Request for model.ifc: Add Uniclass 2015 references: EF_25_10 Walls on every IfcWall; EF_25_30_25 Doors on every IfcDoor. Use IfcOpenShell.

First a look at what the model holds.

```python
import ifcopenshell

model = ifcopenshell.open("model.ifc")
print(model.schema)
print("classifications:", [c.Name for c in model.by_type("IfcClassification")])
for ifc_class in ("IfcDoor", "IfcRoof", "IfcStair", "IfcWall", "IfcWindow"):
    print(ifc_class, len(model.by_type(ifc_class)))
```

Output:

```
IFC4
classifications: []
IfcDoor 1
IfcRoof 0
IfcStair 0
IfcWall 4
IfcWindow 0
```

```python
import ifcopenshell
import ifcopenshell.api.classification

model = ifcopenshell.open("model.ifc")

system = ifcopenshell.api.classification.add_classification(model, classification="Uniclass 2015")

codes = {
    "IfcWall": ("EF_25_10", "Walls"),
    "IfcDoor": ("EF_25_30_25", "Doors"),
}
for ifc_class, (code, name) in codes.items():
    products = model.by_type(ifc_class)
    ifcopenshell.api.classification.add_reference(
        model, products=products, classification=system, identification=code, name=name
    )
    print(code, len(products))

model.write("model_updated.ifc")
```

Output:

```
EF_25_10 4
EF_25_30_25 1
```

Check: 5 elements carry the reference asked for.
